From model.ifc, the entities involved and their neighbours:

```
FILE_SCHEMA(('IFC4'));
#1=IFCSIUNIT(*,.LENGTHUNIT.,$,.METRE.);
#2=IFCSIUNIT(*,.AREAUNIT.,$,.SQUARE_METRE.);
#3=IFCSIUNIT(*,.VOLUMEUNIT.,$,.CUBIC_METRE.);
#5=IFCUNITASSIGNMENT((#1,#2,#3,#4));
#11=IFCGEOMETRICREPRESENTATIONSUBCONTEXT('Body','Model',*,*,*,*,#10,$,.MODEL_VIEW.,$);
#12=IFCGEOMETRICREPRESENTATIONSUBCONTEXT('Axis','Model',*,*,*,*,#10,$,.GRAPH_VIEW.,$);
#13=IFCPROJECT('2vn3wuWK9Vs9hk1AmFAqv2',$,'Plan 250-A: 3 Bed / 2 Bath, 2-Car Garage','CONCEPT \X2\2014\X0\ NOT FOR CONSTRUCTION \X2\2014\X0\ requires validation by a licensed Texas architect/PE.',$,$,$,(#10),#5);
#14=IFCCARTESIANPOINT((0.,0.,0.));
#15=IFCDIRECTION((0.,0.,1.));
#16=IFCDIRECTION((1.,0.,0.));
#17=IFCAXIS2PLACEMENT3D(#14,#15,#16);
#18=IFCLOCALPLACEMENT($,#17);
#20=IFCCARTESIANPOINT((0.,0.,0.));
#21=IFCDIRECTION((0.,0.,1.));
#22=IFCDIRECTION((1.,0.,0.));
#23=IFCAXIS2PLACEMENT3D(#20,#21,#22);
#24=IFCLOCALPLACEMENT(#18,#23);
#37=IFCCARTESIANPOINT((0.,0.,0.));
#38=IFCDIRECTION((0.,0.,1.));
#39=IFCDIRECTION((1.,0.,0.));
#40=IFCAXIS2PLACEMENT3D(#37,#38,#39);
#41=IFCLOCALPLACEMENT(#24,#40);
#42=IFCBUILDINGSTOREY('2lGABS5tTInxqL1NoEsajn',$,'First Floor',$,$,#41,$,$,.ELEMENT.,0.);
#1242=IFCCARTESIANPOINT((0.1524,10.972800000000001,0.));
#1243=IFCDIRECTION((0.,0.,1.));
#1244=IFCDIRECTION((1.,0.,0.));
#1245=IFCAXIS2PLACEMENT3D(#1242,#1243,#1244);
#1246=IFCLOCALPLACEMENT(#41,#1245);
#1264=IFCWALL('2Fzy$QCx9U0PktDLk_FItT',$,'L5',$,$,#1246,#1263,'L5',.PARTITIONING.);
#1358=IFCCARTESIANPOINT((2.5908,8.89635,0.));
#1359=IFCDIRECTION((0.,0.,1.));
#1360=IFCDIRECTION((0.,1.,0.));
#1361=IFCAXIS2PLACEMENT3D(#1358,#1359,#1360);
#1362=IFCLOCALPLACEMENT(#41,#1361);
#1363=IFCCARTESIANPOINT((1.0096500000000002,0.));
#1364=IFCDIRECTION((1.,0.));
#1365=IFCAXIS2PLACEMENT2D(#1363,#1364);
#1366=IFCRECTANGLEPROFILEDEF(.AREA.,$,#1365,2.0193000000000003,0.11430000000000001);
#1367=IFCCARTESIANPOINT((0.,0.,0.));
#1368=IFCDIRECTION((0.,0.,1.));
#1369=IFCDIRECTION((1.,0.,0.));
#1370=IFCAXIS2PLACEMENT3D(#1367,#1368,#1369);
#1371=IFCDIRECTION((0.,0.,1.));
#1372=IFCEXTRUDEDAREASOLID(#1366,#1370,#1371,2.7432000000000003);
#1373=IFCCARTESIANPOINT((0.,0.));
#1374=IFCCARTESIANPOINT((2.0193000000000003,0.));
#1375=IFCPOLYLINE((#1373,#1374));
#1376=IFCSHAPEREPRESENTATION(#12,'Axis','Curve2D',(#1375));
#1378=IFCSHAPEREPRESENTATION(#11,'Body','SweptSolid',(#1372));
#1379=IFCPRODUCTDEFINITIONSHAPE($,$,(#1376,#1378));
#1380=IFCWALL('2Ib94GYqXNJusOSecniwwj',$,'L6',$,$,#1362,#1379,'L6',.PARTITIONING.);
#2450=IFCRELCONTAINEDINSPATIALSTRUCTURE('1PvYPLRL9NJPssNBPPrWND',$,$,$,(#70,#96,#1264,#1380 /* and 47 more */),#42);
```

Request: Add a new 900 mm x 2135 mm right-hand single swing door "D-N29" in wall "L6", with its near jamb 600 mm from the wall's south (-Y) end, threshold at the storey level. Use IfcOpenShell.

```python
import numpy as np
import ifcopenshell
import ifcopenshell.api.feature
import ifcopenshell.api.geometry
import ifcopenshell.api.root
import ifcopenshell.api.spatial
import ifcopenshell.geom
import ifcopenshell.util.element
import ifcopenshell.util.placement
import ifcopenshell.util.representation
import ifcopenshell.util.shape
import ifcopenshell.util.unit

model = ifcopenshell.open("model.ifc")
unit_scale = ifcopenshell.util.unit.calculate_unit_scale(model)
settings = ifcopenshell.geom.settings()


def volume(element):
    """Net volume in cubic metres, openings subtracted."""
    shape = ifcopenshell.geom.create_shape(settings, element)
    return ifcopenshell.util.shape.get_volume(shape.geometry)


wall = model.by_guid("2Ib94GYqXNJusOSecniwwj")
storey = ifcopenshell.util.element.get_container(wall, ifc_class="IfcBuildingStorey")
context = ifcopenshell.util.representation.get_context(model, "Model", "Body", "MODEL_VIEW")
before = volume(wall)

width, height, from_end, sill = 0.9, 2.135, 0.6, 0.0  # metres

# The wall runs along its own X axis, and the end named is its -X end.
wall_shape = ifcopenshell.geom.create_shape(settings, wall)
x, y, z = ifcopenshell.util.shape.get_vertices(wall_shape.geometry).T
start = x.min() + from_end
face, thickness = float(y.min()), float(y.max() - y.min())
wall_matrix = ifcopenshell.util.placement.get_local_placement(wall.ObjectPlacement)
level = ifcopenshell.util.placement.get_local_placement(storey.ObjectPlacement)[2, 3]


def in_wall(x, y):
    """Placement at x, y metres in the wall's axes, at sill height."""
    matrix = wall_matrix.copy()
    matrix[:, 3] = wall_matrix @ np.array([x / unit_scale, y / unit_scale, 0.0, 1.0])
    matrix[2, 3] = level + sill / unit_scale
    return matrix


# Opening: a box that overshoots both wall faces by 50 mm.
opening = ifcopenshell.api.root.create_entity(model, ifc_class="IfcOpeningElement", predefined_type="OPENING")
box = ifcopenshell.api.geometry.add_wall_representation(
    model, context=context, length=width, height=height, thickness=thickness + 0.1
)
ifcopenshell.api.geometry.assign_representation(model, product=opening, representation=box)
ifcopenshell.api.geometry.edit_object_placement(model, product=opening, matrix=in_wall(start, face - 0.05), is_si=False)
ifcopenshell.api.feature.add_feature(model, feature=opening, element=wall)

door = ifcopenshell.api.root.create_entity(model, ifc_class="IfcDoor", name="D-N29", predefined_type="DOOR")
door.OverallWidth, door.OverallHeight = width / unit_scale, height / unit_scale
door.OperationType = "SINGLE_SWING_RIGHT"
body = ifcopenshell.api.geometry.add_door_representation(
    model,
    context=context,
    overall_width=door.OverallWidth,
    overall_height=door.OverallHeight,
    operation_type="SINGLE_SWING_RIGHT",
    lining_properties={"LiningDepth": thickness / unit_scale, "ThresholdDepth": thickness / unit_scale},
)
ifcopenshell.api.geometry.assign_representation(model, product=door, representation=body)
ifcopenshell.api.spatial.assign_container(model, products=[door], relating_structure=storey)
ifcopenshell.api.feature.add_filling(model, opening=opening, element=door)

# The lining spans the wall, so the door starts at the wall face.
ifcopenshell.api.geometry.edit_object_placement(model, product=door, matrix=in_wall(start, face), is_si=False)

after = volume(wall)

print(f"wall volume {before:.3f} -> {after:.3f} m3")

model.write("model_rev.ifc")
```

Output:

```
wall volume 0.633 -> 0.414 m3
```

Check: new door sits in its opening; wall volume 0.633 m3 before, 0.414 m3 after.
